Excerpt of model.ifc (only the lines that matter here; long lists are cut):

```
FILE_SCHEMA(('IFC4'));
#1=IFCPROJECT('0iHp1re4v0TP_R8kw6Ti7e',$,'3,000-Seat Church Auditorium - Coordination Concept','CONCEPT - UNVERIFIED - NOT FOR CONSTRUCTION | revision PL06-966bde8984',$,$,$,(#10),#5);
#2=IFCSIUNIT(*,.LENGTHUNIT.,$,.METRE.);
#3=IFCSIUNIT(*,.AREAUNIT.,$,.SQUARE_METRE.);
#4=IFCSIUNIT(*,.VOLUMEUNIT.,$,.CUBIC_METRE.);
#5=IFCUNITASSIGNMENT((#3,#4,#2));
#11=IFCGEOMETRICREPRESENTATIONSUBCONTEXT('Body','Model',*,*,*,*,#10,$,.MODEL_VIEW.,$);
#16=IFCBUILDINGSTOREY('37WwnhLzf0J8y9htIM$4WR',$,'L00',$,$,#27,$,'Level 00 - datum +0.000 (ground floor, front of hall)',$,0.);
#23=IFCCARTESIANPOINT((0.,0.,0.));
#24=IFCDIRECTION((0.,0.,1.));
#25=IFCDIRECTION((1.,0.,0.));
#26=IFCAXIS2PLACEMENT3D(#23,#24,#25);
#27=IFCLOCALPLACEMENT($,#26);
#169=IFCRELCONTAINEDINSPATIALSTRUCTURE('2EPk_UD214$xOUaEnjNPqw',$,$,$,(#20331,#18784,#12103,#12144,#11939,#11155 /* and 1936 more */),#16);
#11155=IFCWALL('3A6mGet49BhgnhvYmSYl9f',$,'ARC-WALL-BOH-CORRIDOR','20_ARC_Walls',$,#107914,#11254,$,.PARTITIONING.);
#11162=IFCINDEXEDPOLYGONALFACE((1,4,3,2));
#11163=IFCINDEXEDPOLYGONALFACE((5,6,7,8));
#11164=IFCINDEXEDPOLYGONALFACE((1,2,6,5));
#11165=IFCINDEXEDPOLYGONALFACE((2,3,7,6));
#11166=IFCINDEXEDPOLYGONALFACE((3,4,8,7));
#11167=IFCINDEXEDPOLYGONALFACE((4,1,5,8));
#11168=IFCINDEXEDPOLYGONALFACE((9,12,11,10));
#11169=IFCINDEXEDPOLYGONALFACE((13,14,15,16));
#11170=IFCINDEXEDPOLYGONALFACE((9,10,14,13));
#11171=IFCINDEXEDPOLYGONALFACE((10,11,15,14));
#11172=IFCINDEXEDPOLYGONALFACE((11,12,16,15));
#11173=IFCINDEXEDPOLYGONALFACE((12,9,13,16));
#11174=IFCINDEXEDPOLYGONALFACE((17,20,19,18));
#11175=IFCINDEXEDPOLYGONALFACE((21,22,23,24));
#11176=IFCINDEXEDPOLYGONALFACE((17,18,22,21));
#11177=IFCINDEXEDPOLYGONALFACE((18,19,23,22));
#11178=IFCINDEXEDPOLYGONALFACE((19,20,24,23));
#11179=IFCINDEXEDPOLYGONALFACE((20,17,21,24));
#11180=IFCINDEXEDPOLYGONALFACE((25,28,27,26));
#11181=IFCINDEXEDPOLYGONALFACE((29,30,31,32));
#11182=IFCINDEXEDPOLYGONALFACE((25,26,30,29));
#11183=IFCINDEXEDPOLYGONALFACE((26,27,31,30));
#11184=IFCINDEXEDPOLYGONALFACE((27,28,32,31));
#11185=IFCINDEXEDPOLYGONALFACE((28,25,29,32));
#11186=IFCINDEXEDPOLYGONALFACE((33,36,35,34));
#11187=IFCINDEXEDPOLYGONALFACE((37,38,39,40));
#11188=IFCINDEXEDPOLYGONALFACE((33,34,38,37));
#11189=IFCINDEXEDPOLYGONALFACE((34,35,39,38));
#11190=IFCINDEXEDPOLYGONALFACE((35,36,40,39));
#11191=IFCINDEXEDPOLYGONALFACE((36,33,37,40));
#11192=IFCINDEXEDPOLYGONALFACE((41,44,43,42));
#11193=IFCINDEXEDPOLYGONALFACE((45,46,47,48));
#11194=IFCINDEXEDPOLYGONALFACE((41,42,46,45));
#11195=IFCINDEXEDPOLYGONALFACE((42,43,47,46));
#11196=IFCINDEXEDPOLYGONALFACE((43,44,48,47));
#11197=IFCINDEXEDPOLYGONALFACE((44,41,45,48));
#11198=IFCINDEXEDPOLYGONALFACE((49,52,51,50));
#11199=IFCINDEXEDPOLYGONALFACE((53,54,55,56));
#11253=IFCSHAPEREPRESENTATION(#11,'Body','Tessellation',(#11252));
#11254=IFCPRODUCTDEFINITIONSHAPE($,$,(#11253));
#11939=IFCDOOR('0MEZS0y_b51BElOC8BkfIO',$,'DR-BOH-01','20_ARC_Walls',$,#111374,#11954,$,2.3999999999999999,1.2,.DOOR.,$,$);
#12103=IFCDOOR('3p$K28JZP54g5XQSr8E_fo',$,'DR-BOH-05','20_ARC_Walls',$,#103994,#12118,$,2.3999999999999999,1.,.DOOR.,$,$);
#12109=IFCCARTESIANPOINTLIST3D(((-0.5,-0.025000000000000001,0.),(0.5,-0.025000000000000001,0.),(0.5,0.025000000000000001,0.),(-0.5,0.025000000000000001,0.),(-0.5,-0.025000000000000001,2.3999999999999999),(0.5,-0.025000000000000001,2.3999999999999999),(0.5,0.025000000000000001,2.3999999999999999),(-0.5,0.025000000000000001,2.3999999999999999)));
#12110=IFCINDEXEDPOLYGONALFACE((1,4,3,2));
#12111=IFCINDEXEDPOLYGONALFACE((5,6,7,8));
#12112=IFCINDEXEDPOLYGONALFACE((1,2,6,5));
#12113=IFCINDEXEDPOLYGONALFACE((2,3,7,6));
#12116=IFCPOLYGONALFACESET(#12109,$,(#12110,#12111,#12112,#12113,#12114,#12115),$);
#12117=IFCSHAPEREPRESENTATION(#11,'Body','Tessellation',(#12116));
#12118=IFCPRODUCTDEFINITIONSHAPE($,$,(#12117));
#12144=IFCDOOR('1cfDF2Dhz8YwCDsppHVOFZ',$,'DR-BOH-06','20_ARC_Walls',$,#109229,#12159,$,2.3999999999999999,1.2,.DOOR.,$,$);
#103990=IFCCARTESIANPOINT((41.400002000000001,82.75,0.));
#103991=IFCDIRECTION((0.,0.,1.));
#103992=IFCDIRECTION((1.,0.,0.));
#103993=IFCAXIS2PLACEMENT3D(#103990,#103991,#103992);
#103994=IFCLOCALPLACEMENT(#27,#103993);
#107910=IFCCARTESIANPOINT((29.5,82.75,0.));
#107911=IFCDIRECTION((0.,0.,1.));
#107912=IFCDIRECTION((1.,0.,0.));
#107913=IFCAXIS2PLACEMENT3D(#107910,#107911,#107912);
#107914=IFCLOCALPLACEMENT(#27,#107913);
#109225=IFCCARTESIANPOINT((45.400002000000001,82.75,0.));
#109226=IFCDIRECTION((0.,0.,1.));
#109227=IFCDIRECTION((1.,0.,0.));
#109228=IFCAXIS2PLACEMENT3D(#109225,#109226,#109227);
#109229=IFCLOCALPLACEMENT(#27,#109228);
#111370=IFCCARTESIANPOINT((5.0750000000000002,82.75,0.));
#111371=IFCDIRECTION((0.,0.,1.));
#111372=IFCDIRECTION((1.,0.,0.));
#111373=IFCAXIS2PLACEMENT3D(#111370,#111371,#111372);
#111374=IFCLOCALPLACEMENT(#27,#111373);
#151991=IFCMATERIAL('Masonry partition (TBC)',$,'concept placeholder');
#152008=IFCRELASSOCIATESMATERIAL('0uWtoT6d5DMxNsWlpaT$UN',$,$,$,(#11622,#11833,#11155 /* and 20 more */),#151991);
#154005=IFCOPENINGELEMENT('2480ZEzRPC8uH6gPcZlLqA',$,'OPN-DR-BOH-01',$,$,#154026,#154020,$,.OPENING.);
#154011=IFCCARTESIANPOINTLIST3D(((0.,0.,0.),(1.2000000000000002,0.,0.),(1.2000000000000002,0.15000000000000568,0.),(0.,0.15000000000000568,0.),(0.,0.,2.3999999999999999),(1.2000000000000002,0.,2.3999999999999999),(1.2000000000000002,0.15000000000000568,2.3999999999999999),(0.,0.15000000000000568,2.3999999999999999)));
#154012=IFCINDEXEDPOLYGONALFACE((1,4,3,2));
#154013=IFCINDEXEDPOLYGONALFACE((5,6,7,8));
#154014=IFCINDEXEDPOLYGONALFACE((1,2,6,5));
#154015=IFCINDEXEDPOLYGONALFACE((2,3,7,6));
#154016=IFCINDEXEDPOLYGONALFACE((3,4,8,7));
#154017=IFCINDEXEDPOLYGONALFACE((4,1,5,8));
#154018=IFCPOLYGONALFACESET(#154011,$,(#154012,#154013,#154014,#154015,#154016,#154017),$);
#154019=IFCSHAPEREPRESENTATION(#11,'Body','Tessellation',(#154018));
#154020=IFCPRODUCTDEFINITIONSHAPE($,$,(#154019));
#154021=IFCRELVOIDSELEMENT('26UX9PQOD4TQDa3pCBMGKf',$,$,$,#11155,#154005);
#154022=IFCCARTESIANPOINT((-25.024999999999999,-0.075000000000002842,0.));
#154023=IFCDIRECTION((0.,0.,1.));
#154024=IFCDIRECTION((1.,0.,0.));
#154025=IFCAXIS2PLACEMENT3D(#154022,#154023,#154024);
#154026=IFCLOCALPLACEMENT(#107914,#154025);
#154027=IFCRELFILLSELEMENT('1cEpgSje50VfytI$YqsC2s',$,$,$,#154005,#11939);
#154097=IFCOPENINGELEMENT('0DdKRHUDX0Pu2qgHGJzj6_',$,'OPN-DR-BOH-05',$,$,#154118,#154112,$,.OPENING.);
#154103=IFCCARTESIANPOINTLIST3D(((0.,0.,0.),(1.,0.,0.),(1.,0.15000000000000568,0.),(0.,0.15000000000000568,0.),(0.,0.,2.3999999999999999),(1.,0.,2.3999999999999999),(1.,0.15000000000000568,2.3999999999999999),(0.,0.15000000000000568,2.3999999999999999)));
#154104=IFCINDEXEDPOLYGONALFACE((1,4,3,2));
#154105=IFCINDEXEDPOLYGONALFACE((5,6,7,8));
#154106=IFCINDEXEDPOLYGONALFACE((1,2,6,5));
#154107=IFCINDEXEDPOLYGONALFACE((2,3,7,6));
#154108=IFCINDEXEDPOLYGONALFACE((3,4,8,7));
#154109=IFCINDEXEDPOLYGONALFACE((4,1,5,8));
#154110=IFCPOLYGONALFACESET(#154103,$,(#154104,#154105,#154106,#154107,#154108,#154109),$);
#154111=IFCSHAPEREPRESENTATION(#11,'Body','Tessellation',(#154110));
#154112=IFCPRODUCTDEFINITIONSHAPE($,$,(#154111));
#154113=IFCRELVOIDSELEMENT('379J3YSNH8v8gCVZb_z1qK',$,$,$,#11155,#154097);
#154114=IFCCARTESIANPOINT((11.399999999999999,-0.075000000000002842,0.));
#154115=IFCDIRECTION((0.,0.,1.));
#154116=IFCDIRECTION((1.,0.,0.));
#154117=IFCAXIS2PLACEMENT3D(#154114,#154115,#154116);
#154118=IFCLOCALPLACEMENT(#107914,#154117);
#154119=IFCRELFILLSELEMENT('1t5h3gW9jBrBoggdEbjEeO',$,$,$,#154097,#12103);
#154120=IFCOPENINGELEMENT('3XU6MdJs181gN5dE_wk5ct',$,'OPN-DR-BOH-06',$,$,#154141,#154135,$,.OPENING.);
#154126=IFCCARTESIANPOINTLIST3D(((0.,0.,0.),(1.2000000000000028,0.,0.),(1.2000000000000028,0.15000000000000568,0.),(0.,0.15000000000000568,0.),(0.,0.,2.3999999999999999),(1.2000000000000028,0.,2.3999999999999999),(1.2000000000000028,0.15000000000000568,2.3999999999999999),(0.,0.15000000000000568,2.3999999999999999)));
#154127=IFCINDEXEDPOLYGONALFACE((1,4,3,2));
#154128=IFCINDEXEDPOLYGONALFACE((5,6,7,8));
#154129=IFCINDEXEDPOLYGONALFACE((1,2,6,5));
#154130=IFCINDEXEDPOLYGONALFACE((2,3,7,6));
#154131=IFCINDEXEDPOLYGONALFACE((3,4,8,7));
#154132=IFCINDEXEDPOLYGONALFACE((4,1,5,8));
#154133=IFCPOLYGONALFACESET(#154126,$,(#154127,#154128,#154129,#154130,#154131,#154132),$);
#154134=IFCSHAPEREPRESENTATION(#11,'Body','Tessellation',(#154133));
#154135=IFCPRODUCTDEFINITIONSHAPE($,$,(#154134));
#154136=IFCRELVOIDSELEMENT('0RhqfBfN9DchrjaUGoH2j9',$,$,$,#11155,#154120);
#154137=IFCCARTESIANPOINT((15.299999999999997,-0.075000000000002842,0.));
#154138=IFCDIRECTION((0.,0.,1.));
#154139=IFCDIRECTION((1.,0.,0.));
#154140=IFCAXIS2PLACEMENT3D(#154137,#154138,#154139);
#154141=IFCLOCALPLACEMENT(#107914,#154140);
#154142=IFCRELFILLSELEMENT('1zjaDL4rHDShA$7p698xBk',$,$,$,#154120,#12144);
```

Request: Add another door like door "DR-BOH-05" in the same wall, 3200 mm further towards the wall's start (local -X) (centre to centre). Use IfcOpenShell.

```python
import ifcopenshell
import ifcopenshell.api.feature
import ifcopenshell.api.geometry
import ifcopenshell.api.root
import ifcopenshell.geom
import ifcopenshell.util.element
import ifcopenshell.util.placement
import ifcopenshell.util.shape
import ifcopenshell.util.unit

model = ifcopenshell.open("model.ifc")
unit_scale = ifcopenshell.util.unit.calculate_unit_scale(model)
settings = ifcopenshell.geom.settings()


def volume(element):
    """Net volume in cubic metres, openings subtracted."""
    shape = ifcopenshell.geom.create_shape(settings, element)
    return ifcopenshell.util.shape.get_volume(shape.geometry)


door = model.by_guid("3p$K28JZP54g5XQSr8E_fo")
opening = door.FillsVoids[0].RelatingOpeningElement
wall = opening.VoidsElements[0].RelatingBuildingElement
before = volume(wall)
shift = ifcopenshell.util.placement.get_local_placement(wall.ObjectPlacement)[:3, 0] * -3.2 / unit_scale

# copy_class copies the void relationship, type, container and properties, but no geometry.
new_opening = ifcopenshell.api.root.copy_class(model, product=opening)
new_opening.Representation = ifcopenshell.util.element.copy_deep(
    model, opening.Representation, exclude=["IfcGeometricRepresentationContext", "IfcRepresentationMap"]
)
new_door = ifcopenshell.api.root.copy_class(model, product=door)
new_door.Representation = ifcopenshell.util.element.copy_deep(
    model, door.Representation, exclude=["IfcGeometricRepresentationContext", "IfcRepresentationMap"]
)
ifcopenshell.api.feature.add_filling(model, opening=new_opening, element=new_door)

for old, new in ((opening, new_opening), (door, new_door)):
    matrix = ifcopenshell.util.placement.get_local_placement(old.ObjectPlacement)
    matrix[:3, 3] += shift
    ifcopenshell.api.geometry.edit_object_placement(model, product=new, matrix=matrix, is_si=False)

after = volume(wall)

print(f"wall volume {before:.3f} -> {after:.3f} m3")

model.write("model_v2.ifc")
```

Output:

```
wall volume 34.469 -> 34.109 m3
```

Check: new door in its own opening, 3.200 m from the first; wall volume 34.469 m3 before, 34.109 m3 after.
